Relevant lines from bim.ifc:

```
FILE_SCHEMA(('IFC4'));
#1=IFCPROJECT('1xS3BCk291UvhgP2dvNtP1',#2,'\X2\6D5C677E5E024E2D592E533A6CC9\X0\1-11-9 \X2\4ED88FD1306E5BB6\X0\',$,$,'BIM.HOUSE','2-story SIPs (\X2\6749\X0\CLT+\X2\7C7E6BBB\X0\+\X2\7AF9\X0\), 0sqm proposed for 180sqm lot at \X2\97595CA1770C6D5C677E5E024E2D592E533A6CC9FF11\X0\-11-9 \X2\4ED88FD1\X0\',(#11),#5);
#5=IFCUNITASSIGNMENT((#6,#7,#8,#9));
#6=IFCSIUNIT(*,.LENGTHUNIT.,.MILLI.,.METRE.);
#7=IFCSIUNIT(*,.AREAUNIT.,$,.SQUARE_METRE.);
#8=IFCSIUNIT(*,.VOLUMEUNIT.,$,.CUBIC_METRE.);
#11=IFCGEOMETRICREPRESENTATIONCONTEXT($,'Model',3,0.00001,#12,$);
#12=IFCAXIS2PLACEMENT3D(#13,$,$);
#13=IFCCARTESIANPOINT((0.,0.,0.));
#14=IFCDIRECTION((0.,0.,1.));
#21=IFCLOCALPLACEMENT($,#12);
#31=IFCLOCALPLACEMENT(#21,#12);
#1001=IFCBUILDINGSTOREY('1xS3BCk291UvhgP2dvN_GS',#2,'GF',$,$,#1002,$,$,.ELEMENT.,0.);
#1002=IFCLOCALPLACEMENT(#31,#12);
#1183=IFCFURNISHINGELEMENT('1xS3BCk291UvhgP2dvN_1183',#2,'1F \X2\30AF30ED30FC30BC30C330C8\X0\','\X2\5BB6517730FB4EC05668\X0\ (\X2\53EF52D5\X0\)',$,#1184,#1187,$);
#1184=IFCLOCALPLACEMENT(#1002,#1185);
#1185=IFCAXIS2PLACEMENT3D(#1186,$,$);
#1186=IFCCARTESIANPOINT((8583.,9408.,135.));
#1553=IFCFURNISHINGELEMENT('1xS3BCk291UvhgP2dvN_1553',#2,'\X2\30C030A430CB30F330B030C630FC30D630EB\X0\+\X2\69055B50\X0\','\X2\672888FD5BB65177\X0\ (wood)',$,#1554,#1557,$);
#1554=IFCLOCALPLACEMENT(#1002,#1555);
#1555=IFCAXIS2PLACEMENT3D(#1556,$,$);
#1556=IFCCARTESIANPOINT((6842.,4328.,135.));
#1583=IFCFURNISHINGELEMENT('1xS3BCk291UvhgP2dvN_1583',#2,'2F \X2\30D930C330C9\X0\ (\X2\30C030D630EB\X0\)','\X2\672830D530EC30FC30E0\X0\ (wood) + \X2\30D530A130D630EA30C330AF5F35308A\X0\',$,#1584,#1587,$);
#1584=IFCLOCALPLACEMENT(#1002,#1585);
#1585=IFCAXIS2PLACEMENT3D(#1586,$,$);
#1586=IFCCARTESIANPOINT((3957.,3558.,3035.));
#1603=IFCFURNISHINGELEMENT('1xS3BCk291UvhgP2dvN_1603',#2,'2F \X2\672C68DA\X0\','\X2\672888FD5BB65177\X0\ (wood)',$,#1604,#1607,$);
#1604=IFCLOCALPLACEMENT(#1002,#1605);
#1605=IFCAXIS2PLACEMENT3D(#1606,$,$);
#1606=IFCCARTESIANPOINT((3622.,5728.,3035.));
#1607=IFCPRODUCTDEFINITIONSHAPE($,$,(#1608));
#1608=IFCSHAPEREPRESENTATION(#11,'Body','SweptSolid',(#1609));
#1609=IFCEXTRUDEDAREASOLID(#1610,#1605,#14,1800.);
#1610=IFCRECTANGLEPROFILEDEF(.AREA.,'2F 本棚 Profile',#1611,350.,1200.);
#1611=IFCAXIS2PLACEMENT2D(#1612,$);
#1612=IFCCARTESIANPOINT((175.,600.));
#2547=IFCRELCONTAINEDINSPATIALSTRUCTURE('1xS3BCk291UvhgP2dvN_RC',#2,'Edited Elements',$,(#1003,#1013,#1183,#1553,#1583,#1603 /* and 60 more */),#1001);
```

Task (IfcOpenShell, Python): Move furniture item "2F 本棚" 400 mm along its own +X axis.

```python
import ifcopenshell
import ifcopenshell.api.geometry
import ifcopenshell.util.placement
import ifcopenshell.util.unit

model = ifcopenshell.open("bim.ifc")
unit_scale = ifcopenshell.util.unit.calculate_unit_scale(model)

item = model.by_guid("1xS3BCk291UvhgP2dvN_1603")
matrix = ifcopenshell.util.placement.get_local_placement(item.ObjectPlacement)
matrix[:3, 3] += matrix[:3, 0] * 0.4 / unit_scale
ifcopenshell.api.geometry.edit_object_placement(model, product=item, matrix=matrix, is_si=False)

print(ifcopenshell.util.placement.get_local_placement(item.ObjectPlacement).round(3) + 0.0)

model.write("bim-out.ifc")
```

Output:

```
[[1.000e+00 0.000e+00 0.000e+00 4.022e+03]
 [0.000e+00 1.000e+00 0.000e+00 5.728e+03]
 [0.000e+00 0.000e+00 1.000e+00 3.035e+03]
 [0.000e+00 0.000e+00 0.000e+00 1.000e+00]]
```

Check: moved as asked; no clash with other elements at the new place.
